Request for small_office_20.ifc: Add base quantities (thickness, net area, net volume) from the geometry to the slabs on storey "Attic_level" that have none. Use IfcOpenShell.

First a look at what the model holds.

```python
import ifcopenshell
import ifcopenshell.util.element
import ifcopenshell.util.unit

model = ifcopenshell.open("small_office_20.ifc")
print(model.schema)
for unit_type in ("LENGTHUNIT", "AREAUNIT", "VOLUMEUNIT"):
    print(unit_type, ifcopenshell.util.unit.calculate_unit_scale(model, unit_type))
storey = next(s for s in model.by_type("IfcBuildingStorey") if s.Name == "Attic_level")
slabs = [e for e in ifcopenshell.util.element.get_decomposition(storey) if e.is_a("IfcSlab")]
for e in sorted(slabs, key=lambda e: e.id()):
    print(e.id(), e.is_a(), e.Name, list(ifcopenshell.util.element.get_psets(e, qtos_only=True)), sep=" | ")
```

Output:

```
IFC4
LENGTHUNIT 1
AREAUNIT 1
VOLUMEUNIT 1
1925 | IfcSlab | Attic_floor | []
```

```python
import ifcopenshell
import ifcopenshell.api.pset
import ifcopenshell.geom
import ifcopenshell.util.element
import ifcopenshell.util.shape
import ifcopenshell.util.unit

model = ifcopenshell.open("small_office_20.ifc")
unit_scale = ifcopenshell.util.unit.calculate_unit_scale(model)
area_scale = ifcopenshell.util.unit.calculate_unit_scale(model, "AREAUNIT")
volume_scale = ifcopenshell.util.unit.calculate_unit_scale(model, "VOLUMEUNIT")
settings = ifcopenshell.geom.settings()

storey = next(s for s in model.by_type("IfcBuildingStorey") if s.Name == "Attic_level")
slabs = [e for e in ifcopenshell.util.element.get_decomposition(storey) if e.is_a("IfcSlab")]

for e in sorted(slabs, key=lambda e: e.id()):
    if ifcopenshell.util.element.get_psets(e, qtos_only=True, should_inherit=False):
        continue
    # Geometry comes back in metres, in the element's own axes.
    shape = ifcopenshell.geom.create_shape(settings, e)
    values = {
        "Width": ifcopenshell.util.shape.get_z(shape.geometry) / unit_scale,
        "NetArea": ifcopenshell.util.shape.get_footprint_area(shape.geometry) / area_scale,
        "NetVolume": ifcopenshell.util.shape.get_volume(shape.geometry) / volume_scale,
    }
    qto = ifcopenshell.api.pset.add_qto(model, product=e, name="Qto_SlabBaseQuantities")
    ifcopenshell.api.pset.edit_qto(model, qto=qto, properties=values)
    print(e.id(), {k: round(v, 3) for k, v in values.items()})

model.write("small_office_20_edited.ifc")
```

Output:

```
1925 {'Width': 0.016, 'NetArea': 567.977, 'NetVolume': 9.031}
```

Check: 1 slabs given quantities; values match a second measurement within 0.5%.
